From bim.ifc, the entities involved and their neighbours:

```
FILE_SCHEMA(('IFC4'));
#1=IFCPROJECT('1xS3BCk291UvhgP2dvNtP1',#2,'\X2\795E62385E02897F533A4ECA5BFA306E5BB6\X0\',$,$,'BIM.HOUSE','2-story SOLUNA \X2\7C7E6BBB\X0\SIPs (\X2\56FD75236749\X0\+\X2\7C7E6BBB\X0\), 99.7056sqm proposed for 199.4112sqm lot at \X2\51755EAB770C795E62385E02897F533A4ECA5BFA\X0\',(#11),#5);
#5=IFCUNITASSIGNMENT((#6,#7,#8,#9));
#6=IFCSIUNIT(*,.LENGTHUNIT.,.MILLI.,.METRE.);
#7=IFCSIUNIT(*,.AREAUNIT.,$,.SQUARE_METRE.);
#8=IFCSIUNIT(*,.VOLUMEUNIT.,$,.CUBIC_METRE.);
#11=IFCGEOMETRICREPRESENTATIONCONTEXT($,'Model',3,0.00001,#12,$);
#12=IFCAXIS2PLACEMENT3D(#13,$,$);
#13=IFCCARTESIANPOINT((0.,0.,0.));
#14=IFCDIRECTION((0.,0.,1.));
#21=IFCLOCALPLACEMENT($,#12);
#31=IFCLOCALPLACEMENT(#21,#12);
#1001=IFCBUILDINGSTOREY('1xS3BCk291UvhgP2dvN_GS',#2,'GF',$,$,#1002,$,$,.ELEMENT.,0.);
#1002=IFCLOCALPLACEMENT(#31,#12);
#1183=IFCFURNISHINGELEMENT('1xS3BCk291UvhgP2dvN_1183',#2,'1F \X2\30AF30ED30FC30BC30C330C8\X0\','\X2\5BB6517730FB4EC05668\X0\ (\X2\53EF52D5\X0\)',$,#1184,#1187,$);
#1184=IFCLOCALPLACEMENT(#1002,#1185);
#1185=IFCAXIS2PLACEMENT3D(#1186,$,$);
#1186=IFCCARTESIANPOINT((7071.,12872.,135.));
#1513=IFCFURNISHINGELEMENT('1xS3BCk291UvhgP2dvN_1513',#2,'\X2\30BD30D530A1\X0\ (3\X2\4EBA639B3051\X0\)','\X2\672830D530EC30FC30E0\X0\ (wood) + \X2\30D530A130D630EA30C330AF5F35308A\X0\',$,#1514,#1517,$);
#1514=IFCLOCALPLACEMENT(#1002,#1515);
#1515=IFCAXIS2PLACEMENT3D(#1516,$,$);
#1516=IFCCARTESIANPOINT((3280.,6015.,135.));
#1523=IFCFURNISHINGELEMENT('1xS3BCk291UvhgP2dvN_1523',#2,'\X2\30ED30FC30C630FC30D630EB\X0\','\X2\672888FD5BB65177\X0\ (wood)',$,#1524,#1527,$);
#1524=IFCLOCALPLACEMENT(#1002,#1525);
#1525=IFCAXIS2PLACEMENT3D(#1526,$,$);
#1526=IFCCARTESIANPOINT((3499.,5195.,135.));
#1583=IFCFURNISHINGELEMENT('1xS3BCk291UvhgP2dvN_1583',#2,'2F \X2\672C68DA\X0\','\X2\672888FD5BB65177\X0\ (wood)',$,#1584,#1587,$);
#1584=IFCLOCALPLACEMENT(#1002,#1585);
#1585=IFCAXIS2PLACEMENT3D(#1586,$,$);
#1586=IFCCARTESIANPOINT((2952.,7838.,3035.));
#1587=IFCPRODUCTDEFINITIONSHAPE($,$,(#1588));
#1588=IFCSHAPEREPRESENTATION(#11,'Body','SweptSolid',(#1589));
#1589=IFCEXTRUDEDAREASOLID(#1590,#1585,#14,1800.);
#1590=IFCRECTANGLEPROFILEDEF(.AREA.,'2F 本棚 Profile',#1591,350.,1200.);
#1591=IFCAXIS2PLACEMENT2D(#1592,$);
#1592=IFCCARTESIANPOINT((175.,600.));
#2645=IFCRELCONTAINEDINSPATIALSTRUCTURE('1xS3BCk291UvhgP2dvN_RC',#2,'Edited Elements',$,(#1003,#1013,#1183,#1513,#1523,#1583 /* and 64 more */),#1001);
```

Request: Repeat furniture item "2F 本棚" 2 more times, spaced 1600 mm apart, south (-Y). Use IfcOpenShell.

```python
import numpy as np
import ifcopenshell
import ifcopenshell.api.geometry
import ifcopenshell.api.root
import ifcopenshell.util.element
import ifcopenshell.util.placement
import ifcopenshell.util.unit

model = ifcopenshell.open("bim.ifc")
unit_scale = ifcopenshell.util.unit.calculate_unit_scale(model)


def reuse_history(source, copy):
    """copy_class also copies each property set's owner history, people and application; keep the originals."""
    for rel in copy.IsDefinedBy:
        if rel.is_a("IfcRelDefinesByProperties") and (history := rel.RelatingPropertyDefinition.OwnerHistory):
            rel.RelatingPropertyDefinition.OwnerHistory = source.OwnerHistory
            ifcopenshell.util.element.remove_deep2(model, history)


source = model.by_guid("1xS3BCk291UvhgP2dvN_1583")
base = ifcopenshell.util.placement.get_local_placement(source.ObjectPlacement)
step = np.array([0.0, -1.0, 0.0]) * 1.6 / unit_scale

for i in range(1, 3):
    copy = ifcopenshell.api.root.copy_class(model, product=source)
    copy.Representation = ifcopenshell.util.element.copy_deep(
        model, source.Representation, exclude=["IfcGeometricRepresentationContext", "IfcRepresentationMap"]
    )
    reuse_history(source, copy)
    matrix = base.copy()
    matrix[:3, 3] += i * step
    print("added at", matrix[:3, 3].round(3) + 0.0)
    ifcopenshell.api.geometry.edit_object_placement(model, product=copy, matrix=matrix, is_si=False)

model.write("bim_edited.ifc")
```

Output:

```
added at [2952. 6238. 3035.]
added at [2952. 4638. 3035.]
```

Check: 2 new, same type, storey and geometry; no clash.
